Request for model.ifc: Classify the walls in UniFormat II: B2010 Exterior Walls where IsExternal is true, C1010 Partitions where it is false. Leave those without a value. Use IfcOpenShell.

First a look at what the model holds.

```python
import ifcopenshell
import ifcopenshell.util.element

model = ifcopenshell.open("model.ifc")
print(model.schema)
print("classifications:", [c.Name for c in model.by_type("IfcClassification")])
values = [ifcopenshell.util.element.get_pset(e, "Pset_WallCommon", "IsExternal") for e in model.by_type("IfcWall")]
for value in (True, False, None):
    print("IsExternal", value, values.count(value))
```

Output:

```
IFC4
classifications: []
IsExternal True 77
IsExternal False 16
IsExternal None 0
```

```python
import ifcopenshell
import ifcopenshell.api.classification
import ifcopenshell.util.element

model = ifcopenshell.open("model.ifc")

system = ifcopenshell.api.classification.add_classification(model, classification="UniFormat II")

walls = model.by_type("IfcWall")
external = {e: ifcopenshell.util.element.get_pset(e, "Pset_WallCommon", "IsExternal") for e in walls}
for flag, code, name in ((True, "B2010", "Exterior Walls"), (False, "C1010", "Partitions")):
    products = [e for e in walls if external[e] is flag]
    ifcopenshell.api.classification.add_reference(
        model, products=products, classification=system, identification=code, name=name
    )
    print(code, len(products))

model.write("model_updated.ifc")
```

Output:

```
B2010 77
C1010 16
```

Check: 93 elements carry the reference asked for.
